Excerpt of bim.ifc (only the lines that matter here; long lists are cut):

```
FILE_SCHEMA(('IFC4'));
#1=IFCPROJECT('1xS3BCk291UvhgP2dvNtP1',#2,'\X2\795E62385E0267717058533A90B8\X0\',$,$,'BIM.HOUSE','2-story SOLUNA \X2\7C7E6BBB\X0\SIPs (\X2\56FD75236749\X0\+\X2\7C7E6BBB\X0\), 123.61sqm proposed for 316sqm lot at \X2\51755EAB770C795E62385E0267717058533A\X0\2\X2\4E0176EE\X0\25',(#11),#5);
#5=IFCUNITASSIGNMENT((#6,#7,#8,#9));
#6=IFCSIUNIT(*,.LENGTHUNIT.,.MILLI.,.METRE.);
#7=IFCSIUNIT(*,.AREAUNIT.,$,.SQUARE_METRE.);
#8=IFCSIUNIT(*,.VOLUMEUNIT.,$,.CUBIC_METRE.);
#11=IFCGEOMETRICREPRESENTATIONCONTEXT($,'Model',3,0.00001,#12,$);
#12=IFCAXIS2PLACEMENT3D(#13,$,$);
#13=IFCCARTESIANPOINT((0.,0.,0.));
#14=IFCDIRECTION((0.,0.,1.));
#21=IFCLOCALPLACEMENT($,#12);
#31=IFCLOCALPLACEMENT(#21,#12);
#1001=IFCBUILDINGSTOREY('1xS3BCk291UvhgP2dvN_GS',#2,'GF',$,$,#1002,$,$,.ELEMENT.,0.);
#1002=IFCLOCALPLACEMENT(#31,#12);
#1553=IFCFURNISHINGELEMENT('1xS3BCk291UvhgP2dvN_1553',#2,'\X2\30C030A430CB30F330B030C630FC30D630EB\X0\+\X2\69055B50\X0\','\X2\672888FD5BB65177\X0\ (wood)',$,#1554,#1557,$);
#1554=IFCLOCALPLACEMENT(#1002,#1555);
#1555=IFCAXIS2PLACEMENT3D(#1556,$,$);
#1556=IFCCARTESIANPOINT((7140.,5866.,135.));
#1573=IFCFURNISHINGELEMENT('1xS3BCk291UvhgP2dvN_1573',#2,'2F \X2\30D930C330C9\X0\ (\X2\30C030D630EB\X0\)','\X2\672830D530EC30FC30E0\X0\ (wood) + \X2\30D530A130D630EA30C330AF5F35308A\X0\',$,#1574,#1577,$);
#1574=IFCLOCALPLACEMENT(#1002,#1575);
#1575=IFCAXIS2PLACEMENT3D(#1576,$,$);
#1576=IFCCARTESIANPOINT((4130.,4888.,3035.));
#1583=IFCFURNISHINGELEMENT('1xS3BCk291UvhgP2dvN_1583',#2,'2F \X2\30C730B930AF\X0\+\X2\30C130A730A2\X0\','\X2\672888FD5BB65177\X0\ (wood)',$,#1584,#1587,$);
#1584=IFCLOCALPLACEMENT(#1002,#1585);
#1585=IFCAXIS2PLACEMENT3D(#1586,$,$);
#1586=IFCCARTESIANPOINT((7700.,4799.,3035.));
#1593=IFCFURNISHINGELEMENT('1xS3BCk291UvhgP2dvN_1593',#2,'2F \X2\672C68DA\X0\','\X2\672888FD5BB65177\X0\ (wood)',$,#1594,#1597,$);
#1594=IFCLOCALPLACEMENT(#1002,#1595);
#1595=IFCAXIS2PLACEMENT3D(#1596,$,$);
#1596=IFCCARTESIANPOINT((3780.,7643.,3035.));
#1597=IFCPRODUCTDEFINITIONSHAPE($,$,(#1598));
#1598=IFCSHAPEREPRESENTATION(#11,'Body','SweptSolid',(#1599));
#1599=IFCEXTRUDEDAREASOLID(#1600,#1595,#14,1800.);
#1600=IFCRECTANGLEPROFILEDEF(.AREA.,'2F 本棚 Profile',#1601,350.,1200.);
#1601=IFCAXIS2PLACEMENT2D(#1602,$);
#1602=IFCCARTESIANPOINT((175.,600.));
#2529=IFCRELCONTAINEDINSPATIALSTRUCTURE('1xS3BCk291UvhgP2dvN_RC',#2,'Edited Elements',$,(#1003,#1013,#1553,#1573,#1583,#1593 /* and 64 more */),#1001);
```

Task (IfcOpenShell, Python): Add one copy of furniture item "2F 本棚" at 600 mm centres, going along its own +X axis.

```python
import ifcopenshell
import ifcopenshell.api.geometry
import ifcopenshell.api.root
import ifcopenshell.util.element
import ifcopenshell.util.placement

model = ifcopenshell.open("bim.ifc")


def reuse_history(source, copy):
    """copy_class also copies each property set's owner history, people and application; keep the originals."""
    for rel in copy.IsDefinedBy:
        if rel.is_a("IfcRelDefinesByProperties") and (history := rel.RelatingPropertyDefinition.OwnerHistory):
            rel.RelatingPropertyDefinition.OwnerHistory = source.OwnerHistory
            ifcopenshell.util.element.remove_deep2(model, history)


source = model.by_guid("1xS3BCk291UvhgP2dvN_1593")
base = ifcopenshell.util.placement.get_local_placement(source.ObjectPlacement)
step = base[:3, 0] * 600.0

for i in range(1, 2):
    copy = ifcopenshell.api.root.copy_class(model, product=source)
    copy.Representation = ifcopenshell.util.element.copy_deep(
        model, source.Representation, exclude=["IfcGeometricRepresentationContext", "IfcRepresentationMap"]
    )
    reuse_history(source, copy)
    matrix = base.copy()
    matrix[:3, 3] += i * step
    print("added at", matrix[:3, 3].round(3) + 0.0)
    ifcopenshell.api.geometry.edit_object_placement(model, product=copy, matrix=matrix, is_si=False)

model.write("bim-out.ifc")
```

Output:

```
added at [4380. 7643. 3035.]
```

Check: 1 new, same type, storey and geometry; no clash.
